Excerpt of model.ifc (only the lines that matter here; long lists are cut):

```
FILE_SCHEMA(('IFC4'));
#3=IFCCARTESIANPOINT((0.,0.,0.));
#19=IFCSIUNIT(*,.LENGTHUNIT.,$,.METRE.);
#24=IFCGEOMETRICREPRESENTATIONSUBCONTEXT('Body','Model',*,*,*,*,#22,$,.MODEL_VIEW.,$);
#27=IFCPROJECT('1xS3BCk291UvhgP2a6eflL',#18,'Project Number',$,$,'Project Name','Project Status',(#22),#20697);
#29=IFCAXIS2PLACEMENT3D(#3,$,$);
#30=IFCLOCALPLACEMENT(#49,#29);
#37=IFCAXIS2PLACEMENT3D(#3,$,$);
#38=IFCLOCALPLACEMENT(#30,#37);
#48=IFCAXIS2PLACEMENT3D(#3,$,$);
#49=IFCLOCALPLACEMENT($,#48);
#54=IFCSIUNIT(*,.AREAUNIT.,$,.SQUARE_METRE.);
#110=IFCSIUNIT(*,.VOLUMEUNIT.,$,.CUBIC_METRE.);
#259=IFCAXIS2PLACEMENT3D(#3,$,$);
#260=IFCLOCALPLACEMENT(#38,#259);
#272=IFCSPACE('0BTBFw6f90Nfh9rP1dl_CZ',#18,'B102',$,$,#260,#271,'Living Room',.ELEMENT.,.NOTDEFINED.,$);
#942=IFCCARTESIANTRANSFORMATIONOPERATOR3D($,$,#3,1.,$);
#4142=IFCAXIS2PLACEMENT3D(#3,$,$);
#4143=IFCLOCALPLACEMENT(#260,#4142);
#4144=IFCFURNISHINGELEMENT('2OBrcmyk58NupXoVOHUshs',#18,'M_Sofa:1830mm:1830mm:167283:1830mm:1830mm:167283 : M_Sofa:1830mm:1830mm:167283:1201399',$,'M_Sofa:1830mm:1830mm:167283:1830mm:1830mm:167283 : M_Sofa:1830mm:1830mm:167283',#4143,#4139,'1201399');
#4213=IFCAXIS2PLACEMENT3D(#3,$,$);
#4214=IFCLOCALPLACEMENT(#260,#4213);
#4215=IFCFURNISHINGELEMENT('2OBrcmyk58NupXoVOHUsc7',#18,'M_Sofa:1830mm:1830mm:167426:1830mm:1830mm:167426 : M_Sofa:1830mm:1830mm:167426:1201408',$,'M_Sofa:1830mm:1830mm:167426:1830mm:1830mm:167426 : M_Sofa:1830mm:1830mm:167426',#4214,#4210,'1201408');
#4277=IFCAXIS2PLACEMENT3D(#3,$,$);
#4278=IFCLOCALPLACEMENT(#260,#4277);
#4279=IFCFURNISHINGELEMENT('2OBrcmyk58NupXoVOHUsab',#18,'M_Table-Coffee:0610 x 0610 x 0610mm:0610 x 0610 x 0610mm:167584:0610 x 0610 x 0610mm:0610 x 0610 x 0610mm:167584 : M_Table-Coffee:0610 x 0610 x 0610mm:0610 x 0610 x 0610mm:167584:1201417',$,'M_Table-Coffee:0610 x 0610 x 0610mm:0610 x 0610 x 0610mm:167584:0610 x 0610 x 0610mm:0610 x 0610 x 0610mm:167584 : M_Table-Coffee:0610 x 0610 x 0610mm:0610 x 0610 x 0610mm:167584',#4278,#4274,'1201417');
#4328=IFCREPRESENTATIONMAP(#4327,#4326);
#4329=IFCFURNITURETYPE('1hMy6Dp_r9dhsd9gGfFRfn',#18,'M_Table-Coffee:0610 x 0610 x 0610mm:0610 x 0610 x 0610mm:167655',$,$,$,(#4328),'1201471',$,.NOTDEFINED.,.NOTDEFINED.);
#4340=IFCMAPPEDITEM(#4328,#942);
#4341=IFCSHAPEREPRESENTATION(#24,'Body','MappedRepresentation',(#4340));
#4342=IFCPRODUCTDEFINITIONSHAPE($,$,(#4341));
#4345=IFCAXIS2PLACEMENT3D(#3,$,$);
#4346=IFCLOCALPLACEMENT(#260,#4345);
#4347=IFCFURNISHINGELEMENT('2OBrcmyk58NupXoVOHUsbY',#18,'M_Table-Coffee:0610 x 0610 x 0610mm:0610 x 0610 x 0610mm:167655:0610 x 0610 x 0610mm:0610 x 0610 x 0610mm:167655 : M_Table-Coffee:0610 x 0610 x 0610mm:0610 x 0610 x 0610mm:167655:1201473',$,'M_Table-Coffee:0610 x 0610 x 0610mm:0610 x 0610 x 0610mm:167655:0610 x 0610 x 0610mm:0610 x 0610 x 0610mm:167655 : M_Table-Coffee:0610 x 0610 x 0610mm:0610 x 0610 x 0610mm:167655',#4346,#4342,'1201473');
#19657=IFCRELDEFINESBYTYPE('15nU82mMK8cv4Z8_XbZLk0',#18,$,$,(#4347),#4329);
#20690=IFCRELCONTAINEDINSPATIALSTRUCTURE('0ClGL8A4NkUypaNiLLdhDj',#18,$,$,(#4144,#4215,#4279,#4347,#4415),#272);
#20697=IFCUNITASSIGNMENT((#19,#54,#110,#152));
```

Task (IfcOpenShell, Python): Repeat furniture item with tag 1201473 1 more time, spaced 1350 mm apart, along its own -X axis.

```python
import ifcopenshell
import ifcopenshell.api.geometry
import ifcopenshell.api.root
import ifcopenshell.util.element
import ifcopenshell.util.placement

model = ifcopenshell.open("model.ifc")


def reuse_history(source, copy):
    """copy_class also copies each property set's owner history, people and application; keep the originals."""
    for rel in copy.IsDefinedBy:
        if rel.is_a("IfcRelDefinesByProperties") and (history := rel.RelatingPropertyDefinition.OwnerHistory):
            rel.RelatingPropertyDefinition.OwnerHistory = source.OwnerHistory
            ifcopenshell.util.element.remove_deep2(model, history)


source = model.by_id(4347)
base = ifcopenshell.util.placement.get_local_placement(source.ObjectPlacement)
step = -base[:3, 0] * 1.35

for i in range(1, 2):
    copy = ifcopenshell.api.root.copy_class(model, product=source)
    copy.Representation = ifcopenshell.util.element.copy_deep(
        model, source.Representation, exclude=["IfcGeometricRepresentationContext", "IfcRepresentationMap"]
    )
    copy.Name = "M_Table-Coffee:0610 x 0610 x 0610mm:0610 x 0610 x 0610mm:167655:0610 x 0610 x 0610mm:0610 x 0610 x 0610mm:167655 : M_Table-Coffee:0610 x 0610 x 0610mm:0610 x 0610 x 0610mm"
    copy.Tag = None
    reuse_history(source, copy)
    matrix = base.copy()
    matrix[:3, 3] += i * step
    print("added at", matrix[:3, 3].round(3) + 0.0)
    ifcopenshell.api.geometry.edit_object_placement(model, product=copy, matrix=matrix, is_si=False)

model.write("model-out.ifc")
```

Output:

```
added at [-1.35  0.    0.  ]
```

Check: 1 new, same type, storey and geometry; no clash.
